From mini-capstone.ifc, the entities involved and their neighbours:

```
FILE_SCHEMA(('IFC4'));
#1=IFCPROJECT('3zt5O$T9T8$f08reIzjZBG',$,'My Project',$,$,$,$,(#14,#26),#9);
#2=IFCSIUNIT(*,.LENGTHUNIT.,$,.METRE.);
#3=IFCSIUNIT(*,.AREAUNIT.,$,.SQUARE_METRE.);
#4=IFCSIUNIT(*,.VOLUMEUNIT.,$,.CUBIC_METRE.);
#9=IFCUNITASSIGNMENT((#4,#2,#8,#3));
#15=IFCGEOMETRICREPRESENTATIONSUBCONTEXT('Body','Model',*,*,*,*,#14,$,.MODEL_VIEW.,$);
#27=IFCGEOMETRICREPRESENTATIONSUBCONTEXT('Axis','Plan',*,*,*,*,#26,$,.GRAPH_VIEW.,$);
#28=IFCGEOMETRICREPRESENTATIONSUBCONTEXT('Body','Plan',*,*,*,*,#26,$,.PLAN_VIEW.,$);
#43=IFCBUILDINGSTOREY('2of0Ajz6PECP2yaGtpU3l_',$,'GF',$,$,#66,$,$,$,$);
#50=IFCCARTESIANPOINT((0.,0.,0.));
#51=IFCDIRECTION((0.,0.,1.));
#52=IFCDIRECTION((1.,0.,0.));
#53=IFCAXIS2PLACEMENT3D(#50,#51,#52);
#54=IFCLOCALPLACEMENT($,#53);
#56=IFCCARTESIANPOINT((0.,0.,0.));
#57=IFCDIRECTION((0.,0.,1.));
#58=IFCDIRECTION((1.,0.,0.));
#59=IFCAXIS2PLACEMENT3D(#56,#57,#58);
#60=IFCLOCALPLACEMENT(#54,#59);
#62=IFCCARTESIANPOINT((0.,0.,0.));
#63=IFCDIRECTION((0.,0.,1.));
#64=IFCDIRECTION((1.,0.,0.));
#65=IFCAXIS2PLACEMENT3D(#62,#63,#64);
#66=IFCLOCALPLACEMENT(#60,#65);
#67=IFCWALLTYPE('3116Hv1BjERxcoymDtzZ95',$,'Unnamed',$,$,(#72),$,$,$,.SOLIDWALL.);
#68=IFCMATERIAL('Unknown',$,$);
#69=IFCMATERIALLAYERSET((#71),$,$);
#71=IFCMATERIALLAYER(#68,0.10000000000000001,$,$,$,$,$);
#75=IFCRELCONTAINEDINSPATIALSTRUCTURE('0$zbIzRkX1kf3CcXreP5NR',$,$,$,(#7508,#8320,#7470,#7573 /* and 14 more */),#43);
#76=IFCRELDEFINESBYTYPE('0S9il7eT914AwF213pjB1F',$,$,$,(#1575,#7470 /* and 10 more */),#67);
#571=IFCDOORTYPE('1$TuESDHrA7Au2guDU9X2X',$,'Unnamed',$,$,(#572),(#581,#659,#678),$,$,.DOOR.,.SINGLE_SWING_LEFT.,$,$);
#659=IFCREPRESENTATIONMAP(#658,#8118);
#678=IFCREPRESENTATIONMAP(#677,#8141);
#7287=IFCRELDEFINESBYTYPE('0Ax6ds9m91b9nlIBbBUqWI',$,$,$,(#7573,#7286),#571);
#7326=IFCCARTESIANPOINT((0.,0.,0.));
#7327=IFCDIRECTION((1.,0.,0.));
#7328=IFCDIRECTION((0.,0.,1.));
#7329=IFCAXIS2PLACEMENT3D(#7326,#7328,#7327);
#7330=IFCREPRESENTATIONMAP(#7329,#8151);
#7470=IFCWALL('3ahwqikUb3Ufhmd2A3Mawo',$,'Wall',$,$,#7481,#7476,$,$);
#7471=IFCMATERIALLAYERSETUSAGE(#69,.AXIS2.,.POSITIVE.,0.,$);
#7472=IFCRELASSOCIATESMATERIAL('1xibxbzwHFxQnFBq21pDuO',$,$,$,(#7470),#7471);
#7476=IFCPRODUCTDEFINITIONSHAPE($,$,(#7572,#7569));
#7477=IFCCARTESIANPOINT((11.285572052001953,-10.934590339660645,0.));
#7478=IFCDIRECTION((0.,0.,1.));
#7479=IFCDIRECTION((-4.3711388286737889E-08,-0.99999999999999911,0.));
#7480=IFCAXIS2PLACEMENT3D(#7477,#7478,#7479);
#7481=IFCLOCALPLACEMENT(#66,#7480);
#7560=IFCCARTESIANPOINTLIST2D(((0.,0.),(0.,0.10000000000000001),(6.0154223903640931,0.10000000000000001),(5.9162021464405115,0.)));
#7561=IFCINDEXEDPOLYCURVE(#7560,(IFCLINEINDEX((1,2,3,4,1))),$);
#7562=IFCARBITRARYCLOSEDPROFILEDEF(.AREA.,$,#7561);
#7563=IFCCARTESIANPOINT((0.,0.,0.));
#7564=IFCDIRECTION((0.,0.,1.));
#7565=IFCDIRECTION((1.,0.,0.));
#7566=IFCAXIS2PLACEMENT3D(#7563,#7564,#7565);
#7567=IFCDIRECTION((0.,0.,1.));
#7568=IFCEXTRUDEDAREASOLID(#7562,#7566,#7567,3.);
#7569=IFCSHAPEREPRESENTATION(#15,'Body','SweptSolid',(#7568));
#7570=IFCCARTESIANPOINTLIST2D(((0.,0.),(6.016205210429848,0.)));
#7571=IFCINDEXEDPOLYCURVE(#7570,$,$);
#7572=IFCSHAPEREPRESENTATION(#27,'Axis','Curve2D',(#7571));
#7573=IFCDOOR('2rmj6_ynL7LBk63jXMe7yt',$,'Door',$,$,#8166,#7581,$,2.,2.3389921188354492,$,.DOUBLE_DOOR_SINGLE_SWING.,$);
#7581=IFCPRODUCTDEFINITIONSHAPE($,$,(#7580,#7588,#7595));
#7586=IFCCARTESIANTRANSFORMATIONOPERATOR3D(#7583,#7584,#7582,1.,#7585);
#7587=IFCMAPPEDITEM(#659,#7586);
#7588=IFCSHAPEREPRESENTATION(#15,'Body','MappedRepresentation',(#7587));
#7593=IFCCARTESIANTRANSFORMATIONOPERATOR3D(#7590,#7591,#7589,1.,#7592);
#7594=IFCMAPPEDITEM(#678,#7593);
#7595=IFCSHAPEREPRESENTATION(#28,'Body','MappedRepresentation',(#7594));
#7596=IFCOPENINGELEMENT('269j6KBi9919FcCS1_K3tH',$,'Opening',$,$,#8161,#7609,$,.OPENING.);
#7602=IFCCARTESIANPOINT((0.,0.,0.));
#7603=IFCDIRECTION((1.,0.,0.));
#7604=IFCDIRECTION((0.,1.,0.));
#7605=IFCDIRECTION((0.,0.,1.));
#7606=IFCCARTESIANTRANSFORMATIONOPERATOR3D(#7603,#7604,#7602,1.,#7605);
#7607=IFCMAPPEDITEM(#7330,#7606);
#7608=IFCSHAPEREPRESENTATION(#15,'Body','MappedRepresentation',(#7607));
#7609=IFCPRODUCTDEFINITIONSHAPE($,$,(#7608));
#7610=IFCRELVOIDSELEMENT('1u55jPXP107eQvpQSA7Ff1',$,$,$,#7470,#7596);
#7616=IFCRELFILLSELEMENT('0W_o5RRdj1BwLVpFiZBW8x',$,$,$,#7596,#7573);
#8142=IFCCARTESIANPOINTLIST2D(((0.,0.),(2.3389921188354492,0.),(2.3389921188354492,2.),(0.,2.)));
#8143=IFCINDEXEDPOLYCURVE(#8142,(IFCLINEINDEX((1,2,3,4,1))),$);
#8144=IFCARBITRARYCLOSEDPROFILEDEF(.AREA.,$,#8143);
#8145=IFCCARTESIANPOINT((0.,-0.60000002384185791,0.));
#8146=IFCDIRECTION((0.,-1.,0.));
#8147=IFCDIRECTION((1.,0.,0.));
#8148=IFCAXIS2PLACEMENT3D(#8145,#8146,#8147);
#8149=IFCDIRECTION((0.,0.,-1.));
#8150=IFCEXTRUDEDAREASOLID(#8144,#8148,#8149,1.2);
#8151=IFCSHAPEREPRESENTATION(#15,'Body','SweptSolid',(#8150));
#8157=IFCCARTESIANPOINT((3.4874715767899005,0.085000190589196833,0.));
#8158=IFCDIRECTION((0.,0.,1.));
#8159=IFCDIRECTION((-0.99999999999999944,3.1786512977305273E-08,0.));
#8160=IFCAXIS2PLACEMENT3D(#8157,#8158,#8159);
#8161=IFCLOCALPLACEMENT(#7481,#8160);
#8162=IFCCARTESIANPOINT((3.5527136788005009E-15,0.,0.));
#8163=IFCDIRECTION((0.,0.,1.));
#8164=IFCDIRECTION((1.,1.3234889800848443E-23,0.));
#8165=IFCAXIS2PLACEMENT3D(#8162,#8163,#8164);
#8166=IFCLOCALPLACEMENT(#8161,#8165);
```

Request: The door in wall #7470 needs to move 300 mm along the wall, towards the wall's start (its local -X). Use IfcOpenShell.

```python
import ifcopenshell
import ifcopenshell.api.geometry
import ifcopenshell.util.placement

model = ifcopenshell.open("mini-capstone.ifc")

door = model.by_guid("2rmj6_ynL7LBk63jXMe7yt")
opening = door.FillsVoids[0].RelatingOpeningElement
wall = opening.VoidsElements[0].RelatingBuildingElement

wall_matrix = ifcopenshell.util.placement.get_local_placement(wall.ObjectPlacement)
shift = wall_matrix[:3, 0] * -0.3
before = ifcopenshell.util.placement.get_local_placement(door.ObjectPlacement)[:3, 3].copy()

# The door is placed relative to its opening, so it follows when the opening moves.
matrix = ifcopenshell.util.placement.get_local_placement(opening.ObjectPlacement)
matrix[:3, 3] += shift
ifcopenshell.api.geometry.edit_object_placement(
    model, product=opening, matrix=matrix, is_si=False, should_transform_children=True
)

after = ifcopenshell.util.placement.get_local_placement(door.ObjectPlacement)[:3, 3]
print("door moved by", (after - before).round(3) + 0.0)

model.write("mini-capstone_updated.ifc")
```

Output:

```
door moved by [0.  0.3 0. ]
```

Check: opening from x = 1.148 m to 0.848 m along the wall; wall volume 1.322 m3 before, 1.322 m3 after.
